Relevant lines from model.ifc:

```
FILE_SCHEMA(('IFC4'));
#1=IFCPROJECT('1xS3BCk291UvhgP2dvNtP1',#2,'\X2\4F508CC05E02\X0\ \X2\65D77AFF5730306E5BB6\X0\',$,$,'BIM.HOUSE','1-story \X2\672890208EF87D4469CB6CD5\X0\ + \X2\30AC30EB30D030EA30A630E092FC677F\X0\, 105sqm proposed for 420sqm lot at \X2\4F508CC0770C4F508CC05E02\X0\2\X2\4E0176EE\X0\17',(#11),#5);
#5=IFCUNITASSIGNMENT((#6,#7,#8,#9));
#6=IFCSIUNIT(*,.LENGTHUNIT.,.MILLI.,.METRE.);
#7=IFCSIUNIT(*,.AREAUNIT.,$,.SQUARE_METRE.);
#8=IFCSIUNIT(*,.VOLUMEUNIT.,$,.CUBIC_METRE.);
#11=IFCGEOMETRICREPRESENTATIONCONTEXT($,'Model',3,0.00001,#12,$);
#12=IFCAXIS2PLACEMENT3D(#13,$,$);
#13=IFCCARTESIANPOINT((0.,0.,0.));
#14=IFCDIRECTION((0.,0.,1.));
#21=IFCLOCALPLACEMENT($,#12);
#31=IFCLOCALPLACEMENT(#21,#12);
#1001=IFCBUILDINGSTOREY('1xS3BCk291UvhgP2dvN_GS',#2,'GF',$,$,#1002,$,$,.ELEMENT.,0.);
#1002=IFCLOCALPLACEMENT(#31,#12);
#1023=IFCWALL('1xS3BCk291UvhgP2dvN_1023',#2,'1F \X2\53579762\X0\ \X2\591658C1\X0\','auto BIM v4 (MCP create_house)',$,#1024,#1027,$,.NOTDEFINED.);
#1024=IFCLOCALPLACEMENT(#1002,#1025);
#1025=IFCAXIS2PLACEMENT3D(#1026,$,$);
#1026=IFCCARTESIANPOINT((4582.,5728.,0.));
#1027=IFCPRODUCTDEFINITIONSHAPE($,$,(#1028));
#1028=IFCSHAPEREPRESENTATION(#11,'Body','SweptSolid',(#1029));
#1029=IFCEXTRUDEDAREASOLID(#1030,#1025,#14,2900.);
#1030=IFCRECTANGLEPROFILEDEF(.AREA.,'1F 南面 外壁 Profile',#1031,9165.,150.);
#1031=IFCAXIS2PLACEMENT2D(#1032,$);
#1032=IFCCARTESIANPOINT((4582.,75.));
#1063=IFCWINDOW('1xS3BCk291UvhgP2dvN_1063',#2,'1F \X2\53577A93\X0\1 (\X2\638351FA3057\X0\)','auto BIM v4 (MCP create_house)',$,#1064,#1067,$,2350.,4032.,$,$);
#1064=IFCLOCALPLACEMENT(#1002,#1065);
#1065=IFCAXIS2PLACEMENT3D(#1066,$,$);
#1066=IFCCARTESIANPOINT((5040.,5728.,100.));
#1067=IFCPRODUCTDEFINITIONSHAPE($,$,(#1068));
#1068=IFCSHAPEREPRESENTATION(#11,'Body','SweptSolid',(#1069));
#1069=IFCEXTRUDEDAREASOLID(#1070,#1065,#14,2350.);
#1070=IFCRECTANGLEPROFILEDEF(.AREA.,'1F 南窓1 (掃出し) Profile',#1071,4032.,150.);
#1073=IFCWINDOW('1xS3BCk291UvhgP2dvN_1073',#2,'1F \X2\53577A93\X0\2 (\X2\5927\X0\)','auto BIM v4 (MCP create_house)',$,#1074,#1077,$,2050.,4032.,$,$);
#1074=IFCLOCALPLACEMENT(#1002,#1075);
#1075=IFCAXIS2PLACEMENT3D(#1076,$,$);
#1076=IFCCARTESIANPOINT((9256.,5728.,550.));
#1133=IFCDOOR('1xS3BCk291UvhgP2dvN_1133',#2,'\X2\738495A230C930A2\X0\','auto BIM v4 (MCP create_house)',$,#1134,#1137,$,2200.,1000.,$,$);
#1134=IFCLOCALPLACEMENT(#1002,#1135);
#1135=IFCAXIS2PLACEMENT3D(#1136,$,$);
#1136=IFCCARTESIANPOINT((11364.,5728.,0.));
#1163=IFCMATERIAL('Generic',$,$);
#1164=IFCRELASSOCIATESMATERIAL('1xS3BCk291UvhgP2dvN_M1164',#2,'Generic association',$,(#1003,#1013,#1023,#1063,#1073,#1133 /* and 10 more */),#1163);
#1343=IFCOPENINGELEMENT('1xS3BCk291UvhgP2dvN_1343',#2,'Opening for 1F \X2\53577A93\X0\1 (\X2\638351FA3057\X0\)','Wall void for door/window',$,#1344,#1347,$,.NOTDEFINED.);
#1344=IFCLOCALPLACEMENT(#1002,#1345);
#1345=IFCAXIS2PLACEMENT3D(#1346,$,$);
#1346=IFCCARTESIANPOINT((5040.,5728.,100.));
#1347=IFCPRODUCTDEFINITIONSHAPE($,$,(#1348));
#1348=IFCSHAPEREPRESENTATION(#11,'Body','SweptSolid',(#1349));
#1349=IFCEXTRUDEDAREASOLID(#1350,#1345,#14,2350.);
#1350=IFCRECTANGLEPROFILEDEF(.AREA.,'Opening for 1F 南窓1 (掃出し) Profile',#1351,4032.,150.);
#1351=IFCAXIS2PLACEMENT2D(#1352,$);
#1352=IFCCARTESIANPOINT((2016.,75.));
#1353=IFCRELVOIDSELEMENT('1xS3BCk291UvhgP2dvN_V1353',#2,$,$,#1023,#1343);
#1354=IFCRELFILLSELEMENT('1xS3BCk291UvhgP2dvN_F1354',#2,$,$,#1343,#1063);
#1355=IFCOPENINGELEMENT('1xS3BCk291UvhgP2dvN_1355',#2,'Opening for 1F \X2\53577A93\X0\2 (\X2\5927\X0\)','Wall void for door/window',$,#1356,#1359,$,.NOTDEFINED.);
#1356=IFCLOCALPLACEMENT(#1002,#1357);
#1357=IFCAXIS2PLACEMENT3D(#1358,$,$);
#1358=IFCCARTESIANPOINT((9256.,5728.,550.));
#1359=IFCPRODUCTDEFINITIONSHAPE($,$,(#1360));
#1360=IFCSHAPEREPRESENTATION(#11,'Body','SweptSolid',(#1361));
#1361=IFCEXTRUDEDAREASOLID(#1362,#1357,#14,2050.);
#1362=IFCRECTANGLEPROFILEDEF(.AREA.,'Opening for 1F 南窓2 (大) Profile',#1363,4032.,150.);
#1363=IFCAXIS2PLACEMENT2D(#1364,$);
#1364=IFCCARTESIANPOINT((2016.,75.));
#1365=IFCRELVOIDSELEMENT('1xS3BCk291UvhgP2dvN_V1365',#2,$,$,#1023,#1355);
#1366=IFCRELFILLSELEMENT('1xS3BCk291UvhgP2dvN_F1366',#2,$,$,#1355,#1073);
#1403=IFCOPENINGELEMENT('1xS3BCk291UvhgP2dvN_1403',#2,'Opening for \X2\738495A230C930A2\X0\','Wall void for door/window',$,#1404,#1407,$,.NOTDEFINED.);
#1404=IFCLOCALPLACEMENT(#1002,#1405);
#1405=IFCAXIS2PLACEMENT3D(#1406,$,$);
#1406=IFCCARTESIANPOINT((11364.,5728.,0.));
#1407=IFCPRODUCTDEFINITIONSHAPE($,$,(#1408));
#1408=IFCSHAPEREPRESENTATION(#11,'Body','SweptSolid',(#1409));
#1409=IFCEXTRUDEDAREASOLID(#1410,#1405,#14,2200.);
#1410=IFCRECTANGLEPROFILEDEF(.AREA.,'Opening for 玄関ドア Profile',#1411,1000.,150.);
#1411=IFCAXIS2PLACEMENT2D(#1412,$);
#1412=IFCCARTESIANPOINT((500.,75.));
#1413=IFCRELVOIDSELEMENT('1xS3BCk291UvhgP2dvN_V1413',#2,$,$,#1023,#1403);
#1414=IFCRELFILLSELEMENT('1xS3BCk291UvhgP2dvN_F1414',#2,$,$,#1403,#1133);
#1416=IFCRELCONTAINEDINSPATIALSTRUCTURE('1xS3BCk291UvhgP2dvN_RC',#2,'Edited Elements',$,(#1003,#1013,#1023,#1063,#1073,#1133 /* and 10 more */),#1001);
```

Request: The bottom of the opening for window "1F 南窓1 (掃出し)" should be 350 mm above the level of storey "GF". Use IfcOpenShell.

```python
import numpy as np
import ifcopenshell
import ifcopenshell.api.geometry
import ifcopenshell.geom
import ifcopenshell.util.element
import ifcopenshell.util.placement
import ifcopenshell.util.shape
import ifcopenshell.util.unit

model = ifcopenshell.open("model.ifc")
unit_scale = ifcopenshell.util.unit.calculate_unit_scale(model)

window = model.by_guid("1xS3BCk291UvhgP2dvN_1063")
opening = window.FillsVoids[0].RelatingOpeningElement
storey = ifcopenshell.util.element.get_container(window, ifc_class="IfcBuildingStorey")
level = ifcopenshell.util.placement.get_local_placement(storey.ObjectPlacement)[2, 3]

# The opening's origin need not be at the sill, so measure its lowest point.
shape = ifcopenshell.geom.create_shape(ifcopenshell.geom.settings(), opening)
bottom = ifcopenshell.util.shape.get_shape_bottom_elevation(shape, shape.geometry) / unit_scale
dz = level + 0.35 / unit_scale - bottom

shift = np.array([0.0, 0.0, dz])
# The window is not placed relative to its opening, so move both.
for product in (opening, window):
    matrix = ifcopenshell.util.placement.get_local_placement(product.ObjectPlacement)
    matrix[:3, 3] += shift
    ifcopenshell.api.geometry.edit_object_placement(model, product=product, matrix=matrix, is_si=False)

print(f"moved by {dz * unit_scale:+.3f} m")

model.write("model_rev.ifc")
```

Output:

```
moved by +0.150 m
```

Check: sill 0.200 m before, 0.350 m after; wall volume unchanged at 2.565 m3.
